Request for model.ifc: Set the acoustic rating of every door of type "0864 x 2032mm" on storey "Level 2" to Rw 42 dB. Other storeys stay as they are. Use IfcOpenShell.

First a look at what the model holds.

```python
import ifcopenshell
import ifcopenshell.util.element

model = ifcopenshell.open("model.ifc")
print(model.schema)
storey = next(s for s in model.by_type("IfcBuildingStorey") if s.Name == "Level 2")
doors = [e for e in ifcopenshell.util.element.get_decomposition(storey) if e.is_a("IfcDoor")]
seen = {}
for e in doors:
    element_type = ifcopenshell.util.element.get_type(e)
    key = (element_type.Name if element_type != e and element_type else None, ifcopenshell.util.element.get_pset(e, "Pset_DoorCommon", "AcousticRating"))
    seen[key] = seen.get(key, 0) + 1
for (name, value), count in sorted(seen.items(), key=str):
    print(count, "x", name, "|", value)
```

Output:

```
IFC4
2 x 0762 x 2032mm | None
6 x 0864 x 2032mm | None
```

```python
import ifcopenshell
import ifcopenshell.api.pset
import ifcopenshell.util.element

model = ifcopenshell.open("model.ifc")

storey = next(s for s in model.by_type("IfcBuildingStorey") if s.Name == "Level 2")
doors = [e for e in ifcopenshell.util.element.get_decomposition(storey) if e.is_a("IfcDoor")]

count = 0
for e in doors:
    element_type = ifcopenshell.util.element.get_type(e)
    if element_type in (None, e) or element_type.Name != "0864 x 2032mm":
        continue
    # add_pset returns the element's existing set when there is one.
    pset = ifcopenshell.api.pset.add_pset(model, product=e, name="Pset_DoorCommon")
    ifcopenshell.api.pset.edit_pset(model, pset=pset, properties={"AcousticRating": "Rw 42 dB"})
    count += 1

print(count, "doors updated")

model.write("model-out.ifc")
```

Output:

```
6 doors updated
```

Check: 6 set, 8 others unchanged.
